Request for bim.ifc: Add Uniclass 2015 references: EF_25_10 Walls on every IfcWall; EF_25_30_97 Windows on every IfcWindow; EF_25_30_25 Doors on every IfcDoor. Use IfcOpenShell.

First a look at what the model holds.

```python
import ifcopenshell

model = ifcopenshell.open("bim.ifc")
print(model.schema)
print("classifications:", [c.Name for c in model.by_type("IfcClassification")])
for ifc_class in ("IfcDoor", "IfcRoof", "IfcStair", "IfcWall", "IfcWindow"):
    print(ifc_class, len(model.by_type(ifc_class)))
```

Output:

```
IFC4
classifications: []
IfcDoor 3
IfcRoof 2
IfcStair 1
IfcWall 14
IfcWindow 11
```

```python
import ifcopenshell
import ifcopenshell.api.classification

model = ifcopenshell.open("bim.ifc")

system = ifcopenshell.api.classification.add_classification(model, classification="Uniclass 2015")

codes = {
    "IfcWall": ("EF_25_10", "Walls"),
    "IfcWindow": ("EF_25_30_97", "Windows"),
    "IfcDoor": ("EF_25_30_25", "Doors"),
}
for ifc_class, (code, name) in codes.items():
    products = model.by_type(ifc_class)
    ifcopenshell.api.classification.add_reference(
        model, products=products, classification=system, identification=code, name=name
    )
    print(code, len(products))

model.write("bim_updated.ifc")
```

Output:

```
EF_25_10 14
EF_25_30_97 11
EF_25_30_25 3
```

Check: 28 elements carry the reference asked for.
